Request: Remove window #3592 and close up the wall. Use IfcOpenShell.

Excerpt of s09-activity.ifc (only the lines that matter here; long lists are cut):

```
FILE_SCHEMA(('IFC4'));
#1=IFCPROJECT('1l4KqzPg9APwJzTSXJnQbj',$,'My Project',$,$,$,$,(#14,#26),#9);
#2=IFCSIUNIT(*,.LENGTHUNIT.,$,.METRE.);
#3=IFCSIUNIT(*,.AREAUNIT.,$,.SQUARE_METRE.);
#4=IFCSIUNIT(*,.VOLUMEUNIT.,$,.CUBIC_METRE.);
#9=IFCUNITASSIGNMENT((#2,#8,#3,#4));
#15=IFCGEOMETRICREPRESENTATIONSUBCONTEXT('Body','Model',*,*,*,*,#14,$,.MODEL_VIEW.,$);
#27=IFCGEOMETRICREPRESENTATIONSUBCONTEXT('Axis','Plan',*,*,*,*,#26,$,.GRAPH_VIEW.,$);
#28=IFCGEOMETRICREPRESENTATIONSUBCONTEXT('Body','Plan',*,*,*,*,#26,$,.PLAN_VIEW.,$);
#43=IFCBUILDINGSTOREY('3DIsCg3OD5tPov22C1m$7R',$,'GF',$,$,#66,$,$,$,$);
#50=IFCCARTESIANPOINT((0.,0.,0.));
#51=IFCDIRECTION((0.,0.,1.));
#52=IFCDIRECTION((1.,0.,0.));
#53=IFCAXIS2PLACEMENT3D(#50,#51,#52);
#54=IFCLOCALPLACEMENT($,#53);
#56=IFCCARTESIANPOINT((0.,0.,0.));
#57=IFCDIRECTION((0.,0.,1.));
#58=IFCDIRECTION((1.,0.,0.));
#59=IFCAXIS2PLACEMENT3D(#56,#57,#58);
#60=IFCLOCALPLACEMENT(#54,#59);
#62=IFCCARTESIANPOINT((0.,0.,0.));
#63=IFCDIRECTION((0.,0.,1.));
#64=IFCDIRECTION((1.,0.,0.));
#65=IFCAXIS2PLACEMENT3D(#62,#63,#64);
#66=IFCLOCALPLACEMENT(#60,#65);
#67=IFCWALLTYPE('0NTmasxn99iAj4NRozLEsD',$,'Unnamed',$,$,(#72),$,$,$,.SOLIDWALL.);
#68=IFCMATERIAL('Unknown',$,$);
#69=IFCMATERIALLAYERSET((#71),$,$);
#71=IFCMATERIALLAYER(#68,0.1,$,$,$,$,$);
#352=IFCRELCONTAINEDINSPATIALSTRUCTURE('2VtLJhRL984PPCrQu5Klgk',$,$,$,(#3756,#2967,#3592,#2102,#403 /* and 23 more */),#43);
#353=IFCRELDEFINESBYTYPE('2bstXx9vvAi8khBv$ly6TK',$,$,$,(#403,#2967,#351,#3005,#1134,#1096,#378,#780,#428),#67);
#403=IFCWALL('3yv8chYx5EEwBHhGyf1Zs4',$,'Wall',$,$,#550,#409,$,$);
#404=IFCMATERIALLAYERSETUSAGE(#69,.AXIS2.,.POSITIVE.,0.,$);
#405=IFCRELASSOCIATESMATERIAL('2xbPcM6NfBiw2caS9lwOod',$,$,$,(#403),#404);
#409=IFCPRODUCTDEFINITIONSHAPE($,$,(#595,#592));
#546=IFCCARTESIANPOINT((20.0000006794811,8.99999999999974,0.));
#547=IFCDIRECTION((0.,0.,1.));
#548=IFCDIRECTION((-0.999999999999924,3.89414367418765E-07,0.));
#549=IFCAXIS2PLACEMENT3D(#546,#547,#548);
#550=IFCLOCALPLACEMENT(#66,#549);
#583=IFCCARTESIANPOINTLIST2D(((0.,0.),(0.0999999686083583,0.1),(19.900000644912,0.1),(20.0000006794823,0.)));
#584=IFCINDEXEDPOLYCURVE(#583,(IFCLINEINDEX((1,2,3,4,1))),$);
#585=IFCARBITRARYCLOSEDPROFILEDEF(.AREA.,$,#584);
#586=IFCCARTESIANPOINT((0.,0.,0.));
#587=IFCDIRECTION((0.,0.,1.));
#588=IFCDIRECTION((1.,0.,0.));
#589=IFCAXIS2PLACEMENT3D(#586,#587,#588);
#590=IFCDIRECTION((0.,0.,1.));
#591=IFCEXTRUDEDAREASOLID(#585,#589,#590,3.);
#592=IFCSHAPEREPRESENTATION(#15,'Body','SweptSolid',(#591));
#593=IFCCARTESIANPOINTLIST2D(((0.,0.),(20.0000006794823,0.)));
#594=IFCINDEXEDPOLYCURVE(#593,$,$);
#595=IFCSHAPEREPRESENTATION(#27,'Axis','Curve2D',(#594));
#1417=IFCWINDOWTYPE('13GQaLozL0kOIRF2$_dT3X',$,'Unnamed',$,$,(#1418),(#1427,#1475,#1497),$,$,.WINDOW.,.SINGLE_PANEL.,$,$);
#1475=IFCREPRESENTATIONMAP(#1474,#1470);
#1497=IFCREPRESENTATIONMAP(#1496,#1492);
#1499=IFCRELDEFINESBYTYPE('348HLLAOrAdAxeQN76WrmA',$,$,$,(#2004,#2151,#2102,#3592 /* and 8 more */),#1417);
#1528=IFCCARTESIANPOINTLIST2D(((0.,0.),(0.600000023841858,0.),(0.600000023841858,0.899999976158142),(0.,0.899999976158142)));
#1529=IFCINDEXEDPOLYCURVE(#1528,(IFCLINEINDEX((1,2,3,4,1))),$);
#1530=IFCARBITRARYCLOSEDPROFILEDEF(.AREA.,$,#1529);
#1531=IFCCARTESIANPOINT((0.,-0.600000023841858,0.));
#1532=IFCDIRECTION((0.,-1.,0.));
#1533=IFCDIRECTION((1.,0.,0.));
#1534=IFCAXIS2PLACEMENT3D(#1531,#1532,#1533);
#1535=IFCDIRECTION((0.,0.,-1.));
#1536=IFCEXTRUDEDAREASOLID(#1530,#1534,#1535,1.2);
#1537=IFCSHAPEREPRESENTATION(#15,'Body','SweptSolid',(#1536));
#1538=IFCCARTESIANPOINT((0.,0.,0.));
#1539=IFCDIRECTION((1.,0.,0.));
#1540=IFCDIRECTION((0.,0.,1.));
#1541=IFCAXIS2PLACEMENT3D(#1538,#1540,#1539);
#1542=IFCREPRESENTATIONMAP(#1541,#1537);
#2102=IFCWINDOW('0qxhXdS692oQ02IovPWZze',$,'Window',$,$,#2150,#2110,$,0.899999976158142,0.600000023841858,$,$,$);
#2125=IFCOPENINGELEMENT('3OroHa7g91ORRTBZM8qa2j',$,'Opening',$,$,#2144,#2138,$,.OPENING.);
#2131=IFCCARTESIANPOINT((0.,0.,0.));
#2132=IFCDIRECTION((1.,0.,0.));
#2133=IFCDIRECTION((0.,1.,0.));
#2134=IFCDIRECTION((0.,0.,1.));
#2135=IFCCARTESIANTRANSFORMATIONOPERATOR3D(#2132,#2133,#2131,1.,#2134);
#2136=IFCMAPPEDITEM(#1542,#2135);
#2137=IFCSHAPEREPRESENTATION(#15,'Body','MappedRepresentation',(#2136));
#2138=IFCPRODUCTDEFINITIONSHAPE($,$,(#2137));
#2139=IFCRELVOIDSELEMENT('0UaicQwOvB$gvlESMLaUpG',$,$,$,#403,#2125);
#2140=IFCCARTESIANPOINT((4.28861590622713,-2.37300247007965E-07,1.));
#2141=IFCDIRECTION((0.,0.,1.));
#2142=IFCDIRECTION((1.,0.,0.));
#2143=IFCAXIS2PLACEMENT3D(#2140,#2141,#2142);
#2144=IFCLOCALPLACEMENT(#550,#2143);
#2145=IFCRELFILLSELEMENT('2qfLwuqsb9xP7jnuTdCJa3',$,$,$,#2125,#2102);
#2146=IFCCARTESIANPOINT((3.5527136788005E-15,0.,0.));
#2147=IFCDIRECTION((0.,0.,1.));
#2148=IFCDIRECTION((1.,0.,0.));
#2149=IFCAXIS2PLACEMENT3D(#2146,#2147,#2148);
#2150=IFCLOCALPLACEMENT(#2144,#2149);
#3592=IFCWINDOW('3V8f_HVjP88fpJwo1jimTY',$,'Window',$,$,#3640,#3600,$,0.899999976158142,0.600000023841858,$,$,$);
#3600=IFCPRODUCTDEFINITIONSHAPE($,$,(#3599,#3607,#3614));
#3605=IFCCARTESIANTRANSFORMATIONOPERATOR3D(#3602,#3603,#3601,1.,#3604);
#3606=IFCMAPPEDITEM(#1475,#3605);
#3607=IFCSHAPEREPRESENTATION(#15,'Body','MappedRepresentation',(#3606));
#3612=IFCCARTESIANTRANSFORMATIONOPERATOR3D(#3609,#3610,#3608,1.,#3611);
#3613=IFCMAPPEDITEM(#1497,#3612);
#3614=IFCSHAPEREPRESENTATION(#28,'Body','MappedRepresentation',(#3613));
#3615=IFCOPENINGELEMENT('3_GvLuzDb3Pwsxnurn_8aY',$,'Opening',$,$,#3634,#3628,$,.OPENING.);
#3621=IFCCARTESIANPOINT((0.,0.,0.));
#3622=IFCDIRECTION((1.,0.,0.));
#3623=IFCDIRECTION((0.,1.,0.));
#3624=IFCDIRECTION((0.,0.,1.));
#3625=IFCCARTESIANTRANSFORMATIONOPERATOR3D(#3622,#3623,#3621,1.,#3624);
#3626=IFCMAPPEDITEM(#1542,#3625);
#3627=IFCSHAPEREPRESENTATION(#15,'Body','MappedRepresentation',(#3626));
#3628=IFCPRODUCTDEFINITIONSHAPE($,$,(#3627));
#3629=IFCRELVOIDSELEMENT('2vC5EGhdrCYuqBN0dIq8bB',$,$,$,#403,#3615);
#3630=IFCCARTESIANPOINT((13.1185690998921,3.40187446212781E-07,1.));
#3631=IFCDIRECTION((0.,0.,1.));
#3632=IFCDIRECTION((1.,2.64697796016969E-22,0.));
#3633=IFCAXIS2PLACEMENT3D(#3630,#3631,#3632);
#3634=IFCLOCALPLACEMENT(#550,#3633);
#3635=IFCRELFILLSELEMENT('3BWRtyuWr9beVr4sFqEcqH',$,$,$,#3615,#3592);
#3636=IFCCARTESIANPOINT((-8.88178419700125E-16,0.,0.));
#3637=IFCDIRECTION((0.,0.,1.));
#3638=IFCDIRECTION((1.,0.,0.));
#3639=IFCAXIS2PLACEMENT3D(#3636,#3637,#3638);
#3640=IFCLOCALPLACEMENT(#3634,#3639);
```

```python
import ifcopenshell
import ifcopenshell.api.feature
import ifcopenshell.api.root
import ifcopenshell.geom
import ifcopenshell.util.shape

model = ifcopenshell.open("s09-activity.ifc")
settings = ifcopenshell.geom.settings()


def volume(element):
    """Net volume in cubic metres, openings subtracted."""
    shape = ifcopenshell.geom.create_shape(settings, element)
    return ifcopenshell.util.shape.get_volume(shape.geometry)


window = model.by_guid("3V8f_HVjP88fpJwo1jimTY")
opening = window.FillsVoids[0].RelatingOpeningElement
wall = opening.VoidsElements[0].RelatingBuildingElement
before = volume(wall)

ifcopenshell.api.root.remove_product(model, product=window)
ifcopenshell.api.feature.remove_feature(model, feature=opening)

after = volume(wall)

print(f"wall volume {before:.3f} -> {after:.3f} m3")

model.write("s09-activity_edited.ifc")
```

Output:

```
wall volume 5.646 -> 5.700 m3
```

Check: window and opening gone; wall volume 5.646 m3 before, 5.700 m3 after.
